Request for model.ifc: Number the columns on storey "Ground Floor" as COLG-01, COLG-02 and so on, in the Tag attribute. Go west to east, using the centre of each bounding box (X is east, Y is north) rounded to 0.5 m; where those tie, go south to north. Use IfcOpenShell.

First a look at what the model holds.

```python
import ifcopenshell
import ifcopenshell.util.element
import ifcopenshell.util.placement

model = ifcopenshell.open("model.ifc")
print(model.schema)
storey = next(s for s in model.by_type("IfcBuildingStorey") if s.Name == "Ground Floor")
columns = [e for e in ifcopenshell.util.element.get_decomposition(storey) if e.is_a("IfcColumn")]
for e in sorted(columns, key=lambda e: e.id()):
    origin = ifcopenshell.util.placement.get_local_placement(e.ObjectPlacement)[:3, 3]
    print(e.id(), e.Tag, e.Name, origin.round(2) + 0.0, sep=" | ")
```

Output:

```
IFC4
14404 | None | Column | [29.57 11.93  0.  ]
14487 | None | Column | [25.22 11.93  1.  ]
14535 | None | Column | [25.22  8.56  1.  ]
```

```python
import ifcopenshell
import ifcopenshell.geom
import ifcopenshell.util.element
import ifcopenshell.util.shape

model = ifcopenshell.open("model.ifc")
settings = ifcopenshell.geom.settings()
settings.set("use-world-coords", True)


def centre(element):
    shape = ifcopenshell.geom.create_shape(settings, element)
    return ifcopenshell.util.shape.get_bbox_centroid(shape.geometry)


storey = next(s for s in model.by_type("IfcBuildingStorey") if s.Name == "Ground Floor")
columns = [e for e in ifcopenshell.util.element.get_decomposition(storey) if e.is_a("IfcColumn")]

# Insertion points can sit at a corner or the storey origin, so sort by the geometry (in metres).
centres = {e: centre(e) for e in columns}
columns.sort(key=lambda e: (round(centres[e][0] / 0.5), centres[e][1]))

for i, e in enumerate(columns, start=1):
    number = f"COLG-{i:02d}"
    e.Tag = number
    print(e.id(), number)

model.write("model_updated.ifc")
```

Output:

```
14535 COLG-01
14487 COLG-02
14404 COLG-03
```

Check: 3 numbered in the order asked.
